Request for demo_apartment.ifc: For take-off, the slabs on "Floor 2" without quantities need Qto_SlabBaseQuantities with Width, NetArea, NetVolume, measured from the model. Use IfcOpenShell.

First a look at what the model holds.

```python
import ifcopenshell
import ifcopenshell.util.element
import ifcopenshell.util.unit

model = ifcopenshell.open("demo_apartment.ifc")
print(model.schema)
for unit_type in ("LENGTHUNIT", "AREAUNIT", "VOLUMEUNIT"):
    print(unit_type, ifcopenshell.util.unit.calculate_unit_scale(model, unit_type))
storey = next(s for s in model.by_type("IfcBuildingStorey") if s.Name == "Floor 2")
slabs = [e for e in ifcopenshell.util.element.get_decomposition(storey) if e.is_a("IfcSlab")]
for e in sorted(slabs, key=lambda e: e.id()):
    print(e.id(), e.is_a(), e.Name, list(ifcopenshell.util.element.get_psets(e, qtos_only=True)), sep=" | ")
```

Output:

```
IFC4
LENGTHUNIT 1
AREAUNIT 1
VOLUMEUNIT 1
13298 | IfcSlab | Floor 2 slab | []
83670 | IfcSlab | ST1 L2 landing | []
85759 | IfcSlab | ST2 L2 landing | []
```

```python
import ifcopenshell
import ifcopenshell.api.pset
import ifcopenshell.geom
import ifcopenshell.util.element
import ifcopenshell.util.shape
import ifcopenshell.util.unit

model = ifcopenshell.open("demo_apartment.ifc")
unit_scale = ifcopenshell.util.unit.calculate_unit_scale(model)
area_scale = ifcopenshell.util.unit.calculate_unit_scale(model, "AREAUNIT")
volume_scale = ifcopenshell.util.unit.calculate_unit_scale(model, "VOLUMEUNIT")
settings = ifcopenshell.geom.settings()

storey = next(s for s in model.by_type("IfcBuildingStorey") if s.Name == "Floor 2")
slabs = [e for e in ifcopenshell.util.element.get_decomposition(storey) if e.is_a("IfcSlab")]

for e in sorted(slabs, key=lambda e: e.id()):
    if ifcopenshell.util.element.get_psets(e, qtos_only=True, should_inherit=False):
        continue
    # Geometry comes back in metres, in the element's own axes.
    shape = ifcopenshell.geom.create_shape(settings, e)
    values = {
        "Width": ifcopenshell.util.shape.get_z(shape.geometry) / unit_scale,
        "NetArea": ifcopenshell.util.shape.get_footprint_area(shape.geometry) / area_scale,
        "NetVolume": ifcopenshell.util.shape.get_volume(shape.geometry) / volume_scale,
    }
    qto = ifcopenshell.api.pset.add_qto(model, product=e, name="Qto_SlabBaseQuantities")
    ifcopenshell.api.pset.edit_qto(model, qto=qto, properties=values)
    print(e.id(), {k: round(v, 3) for k, v in values.items()})

model.write("demo_apartment_rev.ifc")
```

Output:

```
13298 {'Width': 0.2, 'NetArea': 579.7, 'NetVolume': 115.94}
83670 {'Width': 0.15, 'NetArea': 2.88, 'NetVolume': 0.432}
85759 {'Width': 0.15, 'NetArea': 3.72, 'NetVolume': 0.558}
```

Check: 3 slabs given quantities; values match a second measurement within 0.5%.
